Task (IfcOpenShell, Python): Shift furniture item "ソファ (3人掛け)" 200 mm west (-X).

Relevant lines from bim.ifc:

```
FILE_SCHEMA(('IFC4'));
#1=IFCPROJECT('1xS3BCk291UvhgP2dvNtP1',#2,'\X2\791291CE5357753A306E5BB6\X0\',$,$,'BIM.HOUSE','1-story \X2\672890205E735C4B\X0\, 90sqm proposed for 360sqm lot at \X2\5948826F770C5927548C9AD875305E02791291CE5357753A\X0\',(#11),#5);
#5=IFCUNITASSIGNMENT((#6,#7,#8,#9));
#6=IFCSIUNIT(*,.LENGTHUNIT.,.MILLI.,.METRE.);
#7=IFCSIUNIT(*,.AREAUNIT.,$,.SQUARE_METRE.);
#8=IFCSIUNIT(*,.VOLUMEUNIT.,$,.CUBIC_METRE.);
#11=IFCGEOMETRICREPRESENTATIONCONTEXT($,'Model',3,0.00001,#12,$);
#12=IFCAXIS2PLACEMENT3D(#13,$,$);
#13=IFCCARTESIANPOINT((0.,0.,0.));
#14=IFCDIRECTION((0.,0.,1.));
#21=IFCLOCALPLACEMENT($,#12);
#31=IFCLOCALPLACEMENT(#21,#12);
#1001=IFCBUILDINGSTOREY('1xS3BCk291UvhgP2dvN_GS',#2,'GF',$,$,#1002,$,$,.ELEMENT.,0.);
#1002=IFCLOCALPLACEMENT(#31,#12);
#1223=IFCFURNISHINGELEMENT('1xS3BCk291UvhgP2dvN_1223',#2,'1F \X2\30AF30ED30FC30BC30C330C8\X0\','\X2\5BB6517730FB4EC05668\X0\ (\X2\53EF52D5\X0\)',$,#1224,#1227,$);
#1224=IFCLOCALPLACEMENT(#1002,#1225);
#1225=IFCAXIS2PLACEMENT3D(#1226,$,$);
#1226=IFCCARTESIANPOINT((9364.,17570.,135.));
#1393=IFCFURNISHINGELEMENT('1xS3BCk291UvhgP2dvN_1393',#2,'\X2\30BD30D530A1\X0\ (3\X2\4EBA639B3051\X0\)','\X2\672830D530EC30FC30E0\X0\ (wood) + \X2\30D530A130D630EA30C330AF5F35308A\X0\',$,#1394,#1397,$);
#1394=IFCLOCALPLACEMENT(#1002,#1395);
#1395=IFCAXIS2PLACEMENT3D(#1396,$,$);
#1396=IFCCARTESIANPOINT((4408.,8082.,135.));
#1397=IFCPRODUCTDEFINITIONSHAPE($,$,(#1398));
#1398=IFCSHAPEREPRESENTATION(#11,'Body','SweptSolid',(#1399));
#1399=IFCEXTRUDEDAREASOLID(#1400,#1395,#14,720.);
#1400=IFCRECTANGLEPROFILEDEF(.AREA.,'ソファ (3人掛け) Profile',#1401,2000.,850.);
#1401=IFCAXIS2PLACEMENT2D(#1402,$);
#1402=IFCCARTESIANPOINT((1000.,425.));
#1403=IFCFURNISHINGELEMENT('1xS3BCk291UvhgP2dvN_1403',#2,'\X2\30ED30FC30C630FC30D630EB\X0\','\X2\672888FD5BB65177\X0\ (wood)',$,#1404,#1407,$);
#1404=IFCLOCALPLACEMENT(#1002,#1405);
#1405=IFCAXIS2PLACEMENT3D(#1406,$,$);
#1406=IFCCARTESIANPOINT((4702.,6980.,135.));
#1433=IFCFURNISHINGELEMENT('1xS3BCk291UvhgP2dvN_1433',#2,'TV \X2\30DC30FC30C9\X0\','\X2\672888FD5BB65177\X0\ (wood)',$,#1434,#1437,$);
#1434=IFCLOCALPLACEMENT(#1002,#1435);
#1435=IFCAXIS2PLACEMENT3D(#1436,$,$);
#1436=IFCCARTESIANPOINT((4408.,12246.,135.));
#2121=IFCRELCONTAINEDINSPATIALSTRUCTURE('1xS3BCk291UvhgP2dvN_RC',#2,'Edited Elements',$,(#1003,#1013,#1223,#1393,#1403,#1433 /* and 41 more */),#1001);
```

```python
import ifcopenshell
import ifcopenshell.api.geometry
import ifcopenshell.util.placement
import ifcopenshell.util.unit

model = ifcopenshell.open("bim.ifc")
unit_scale = ifcopenshell.util.unit.calculate_unit_scale(model)

item = model.by_guid("1xS3BCk291UvhgP2dvN_1393")
matrix = ifcopenshell.util.placement.get_local_placement(item.ObjectPlacement)
matrix[0, 3] -= 0.2 / unit_scale
ifcopenshell.api.geometry.edit_object_placement(model, product=item, matrix=matrix, is_si=False)

print(ifcopenshell.util.placement.get_local_placement(item.ObjectPlacement).round(3) + 0.0)

model.write("bim_updated.ifc")
```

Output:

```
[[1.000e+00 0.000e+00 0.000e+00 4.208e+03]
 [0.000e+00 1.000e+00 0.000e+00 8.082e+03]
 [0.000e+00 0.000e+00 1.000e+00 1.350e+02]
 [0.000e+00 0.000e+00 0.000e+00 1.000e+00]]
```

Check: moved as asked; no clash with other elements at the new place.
